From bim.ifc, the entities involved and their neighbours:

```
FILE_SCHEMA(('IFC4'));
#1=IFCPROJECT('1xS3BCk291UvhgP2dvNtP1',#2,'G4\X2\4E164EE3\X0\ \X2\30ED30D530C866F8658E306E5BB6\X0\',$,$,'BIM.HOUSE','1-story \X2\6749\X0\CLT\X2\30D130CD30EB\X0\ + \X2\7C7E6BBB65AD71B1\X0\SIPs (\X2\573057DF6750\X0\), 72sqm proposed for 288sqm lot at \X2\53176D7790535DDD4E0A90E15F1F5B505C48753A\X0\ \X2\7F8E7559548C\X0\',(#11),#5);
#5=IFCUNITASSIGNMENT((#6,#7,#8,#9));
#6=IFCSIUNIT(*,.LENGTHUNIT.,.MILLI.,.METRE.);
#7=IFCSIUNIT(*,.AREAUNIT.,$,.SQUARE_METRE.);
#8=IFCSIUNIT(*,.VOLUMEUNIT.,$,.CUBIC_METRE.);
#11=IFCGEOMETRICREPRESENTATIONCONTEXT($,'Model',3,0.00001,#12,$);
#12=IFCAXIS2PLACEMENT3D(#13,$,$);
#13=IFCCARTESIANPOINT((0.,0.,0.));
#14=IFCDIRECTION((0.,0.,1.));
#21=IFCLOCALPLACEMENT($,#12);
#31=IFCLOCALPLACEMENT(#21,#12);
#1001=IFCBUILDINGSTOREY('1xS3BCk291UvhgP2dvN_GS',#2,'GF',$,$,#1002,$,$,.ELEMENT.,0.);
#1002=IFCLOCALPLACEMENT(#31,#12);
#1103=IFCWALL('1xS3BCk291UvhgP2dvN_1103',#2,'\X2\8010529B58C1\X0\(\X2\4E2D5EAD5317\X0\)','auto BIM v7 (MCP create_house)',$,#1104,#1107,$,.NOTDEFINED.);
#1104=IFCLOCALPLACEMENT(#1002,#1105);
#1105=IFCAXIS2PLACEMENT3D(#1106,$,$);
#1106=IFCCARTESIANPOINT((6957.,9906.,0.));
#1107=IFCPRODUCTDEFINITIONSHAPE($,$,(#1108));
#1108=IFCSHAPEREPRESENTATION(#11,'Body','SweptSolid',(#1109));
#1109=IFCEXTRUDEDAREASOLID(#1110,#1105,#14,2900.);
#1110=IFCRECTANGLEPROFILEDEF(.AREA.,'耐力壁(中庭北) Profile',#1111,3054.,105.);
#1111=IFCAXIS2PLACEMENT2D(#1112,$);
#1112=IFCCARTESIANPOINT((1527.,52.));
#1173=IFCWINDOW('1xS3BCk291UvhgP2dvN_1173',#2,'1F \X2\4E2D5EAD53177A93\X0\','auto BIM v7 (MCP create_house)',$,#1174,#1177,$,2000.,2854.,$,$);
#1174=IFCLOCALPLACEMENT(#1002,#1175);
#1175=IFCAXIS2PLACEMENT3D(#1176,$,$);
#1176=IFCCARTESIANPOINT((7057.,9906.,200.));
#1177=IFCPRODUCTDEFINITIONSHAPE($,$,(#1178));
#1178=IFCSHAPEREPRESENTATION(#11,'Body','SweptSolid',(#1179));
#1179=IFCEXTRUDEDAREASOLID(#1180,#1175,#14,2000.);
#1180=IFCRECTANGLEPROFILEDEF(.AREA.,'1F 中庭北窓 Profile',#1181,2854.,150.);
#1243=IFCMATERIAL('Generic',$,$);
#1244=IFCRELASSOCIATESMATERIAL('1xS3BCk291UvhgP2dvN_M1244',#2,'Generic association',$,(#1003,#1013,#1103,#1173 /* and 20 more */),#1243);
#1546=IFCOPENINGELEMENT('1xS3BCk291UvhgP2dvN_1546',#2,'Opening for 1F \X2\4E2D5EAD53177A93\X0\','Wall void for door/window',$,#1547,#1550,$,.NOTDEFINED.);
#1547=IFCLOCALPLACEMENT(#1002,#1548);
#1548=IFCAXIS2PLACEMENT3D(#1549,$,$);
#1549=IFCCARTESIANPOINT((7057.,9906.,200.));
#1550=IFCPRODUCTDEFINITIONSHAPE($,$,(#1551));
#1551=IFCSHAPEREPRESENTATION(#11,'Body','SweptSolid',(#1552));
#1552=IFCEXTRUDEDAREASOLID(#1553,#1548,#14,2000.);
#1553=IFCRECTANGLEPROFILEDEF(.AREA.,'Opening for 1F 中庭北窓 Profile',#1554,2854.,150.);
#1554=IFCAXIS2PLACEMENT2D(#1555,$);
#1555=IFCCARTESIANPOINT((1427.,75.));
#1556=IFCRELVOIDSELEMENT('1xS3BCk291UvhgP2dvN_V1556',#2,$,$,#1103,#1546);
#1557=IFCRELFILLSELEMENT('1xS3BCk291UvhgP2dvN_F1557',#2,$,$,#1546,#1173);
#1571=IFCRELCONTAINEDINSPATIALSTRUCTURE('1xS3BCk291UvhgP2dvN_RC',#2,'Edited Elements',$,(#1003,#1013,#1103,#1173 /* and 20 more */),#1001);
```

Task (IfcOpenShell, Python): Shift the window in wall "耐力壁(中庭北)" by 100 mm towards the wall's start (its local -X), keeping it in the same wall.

```python
import ifcopenshell
import ifcopenshell.api.geometry
import ifcopenshell.util.placement
import ifcopenshell.util.unit

model = ifcopenshell.open("bim.ifc")
unit_scale = ifcopenshell.util.unit.calculate_unit_scale(model)

window = model.by_id(1173)
opening = window.FillsVoids[0].RelatingOpeningElement
wall = opening.VoidsElements[0].RelatingBuildingElement

wall_matrix = ifcopenshell.util.placement.get_local_placement(wall.ObjectPlacement)
shift = wall_matrix[:3, 0] * -0.1 / unit_scale
before = ifcopenshell.util.placement.get_local_placement(window.ObjectPlacement)[:3, 3].copy()

# The window is not placed relative to its opening, so move both.
for product in (opening, window):
    matrix = ifcopenshell.util.placement.get_local_placement(product.ObjectPlacement)
    matrix[:3, 3] += shift
    ifcopenshell.api.geometry.edit_object_placement(model, product=product, matrix=matrix, is_si=False)

after = ifcopenshell.util.placement.get_local_placement(window.ObjectPlacement)[:3, 3]
print("window moved by", (after - before).round(3) + 0.0)

model.write("bim-out.ifc")
```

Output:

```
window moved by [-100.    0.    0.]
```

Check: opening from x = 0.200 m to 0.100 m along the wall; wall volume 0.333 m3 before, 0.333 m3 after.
